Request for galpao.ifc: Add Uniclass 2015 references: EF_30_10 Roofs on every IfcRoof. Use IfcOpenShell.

First a look at what the model holds.

```python
import ifcopenshell

model = ifcopenshell.open("galpao.ifc")
print(model.schema)
print("classifications:", [c.Name for c in model.by_type("IfcClassification")])
for ifc_class in ("IfcDoor", "IfcRoof", "IfcStair", "IfcWall", "IfcWindow"):
    print(ifc_class, len(model.by_type(ifc_class)))
```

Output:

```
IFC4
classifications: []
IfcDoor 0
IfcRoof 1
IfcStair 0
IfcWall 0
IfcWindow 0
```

```python
import ifcopenshell
import ifcopenshell.api.classification

model = ifcopenshell.open("galpao.ifc")

system = ifcopenshell.api.classification.add_classification(model, classification="Uniclass 2015")

codes = {
    "IfcRoof": ("EF_30_10", "Roofs"),
}
for ifc_class, (code, name) in codes.items():
    products = model.by_type(ifc_class)
    ifcopenshell.api.classification.add_reference(
        model, products=products, classification=system, identification=code, name=name
    )
    print(code, len(products))

model.write("galpao_v2.ifc")
```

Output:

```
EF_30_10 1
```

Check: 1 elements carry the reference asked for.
